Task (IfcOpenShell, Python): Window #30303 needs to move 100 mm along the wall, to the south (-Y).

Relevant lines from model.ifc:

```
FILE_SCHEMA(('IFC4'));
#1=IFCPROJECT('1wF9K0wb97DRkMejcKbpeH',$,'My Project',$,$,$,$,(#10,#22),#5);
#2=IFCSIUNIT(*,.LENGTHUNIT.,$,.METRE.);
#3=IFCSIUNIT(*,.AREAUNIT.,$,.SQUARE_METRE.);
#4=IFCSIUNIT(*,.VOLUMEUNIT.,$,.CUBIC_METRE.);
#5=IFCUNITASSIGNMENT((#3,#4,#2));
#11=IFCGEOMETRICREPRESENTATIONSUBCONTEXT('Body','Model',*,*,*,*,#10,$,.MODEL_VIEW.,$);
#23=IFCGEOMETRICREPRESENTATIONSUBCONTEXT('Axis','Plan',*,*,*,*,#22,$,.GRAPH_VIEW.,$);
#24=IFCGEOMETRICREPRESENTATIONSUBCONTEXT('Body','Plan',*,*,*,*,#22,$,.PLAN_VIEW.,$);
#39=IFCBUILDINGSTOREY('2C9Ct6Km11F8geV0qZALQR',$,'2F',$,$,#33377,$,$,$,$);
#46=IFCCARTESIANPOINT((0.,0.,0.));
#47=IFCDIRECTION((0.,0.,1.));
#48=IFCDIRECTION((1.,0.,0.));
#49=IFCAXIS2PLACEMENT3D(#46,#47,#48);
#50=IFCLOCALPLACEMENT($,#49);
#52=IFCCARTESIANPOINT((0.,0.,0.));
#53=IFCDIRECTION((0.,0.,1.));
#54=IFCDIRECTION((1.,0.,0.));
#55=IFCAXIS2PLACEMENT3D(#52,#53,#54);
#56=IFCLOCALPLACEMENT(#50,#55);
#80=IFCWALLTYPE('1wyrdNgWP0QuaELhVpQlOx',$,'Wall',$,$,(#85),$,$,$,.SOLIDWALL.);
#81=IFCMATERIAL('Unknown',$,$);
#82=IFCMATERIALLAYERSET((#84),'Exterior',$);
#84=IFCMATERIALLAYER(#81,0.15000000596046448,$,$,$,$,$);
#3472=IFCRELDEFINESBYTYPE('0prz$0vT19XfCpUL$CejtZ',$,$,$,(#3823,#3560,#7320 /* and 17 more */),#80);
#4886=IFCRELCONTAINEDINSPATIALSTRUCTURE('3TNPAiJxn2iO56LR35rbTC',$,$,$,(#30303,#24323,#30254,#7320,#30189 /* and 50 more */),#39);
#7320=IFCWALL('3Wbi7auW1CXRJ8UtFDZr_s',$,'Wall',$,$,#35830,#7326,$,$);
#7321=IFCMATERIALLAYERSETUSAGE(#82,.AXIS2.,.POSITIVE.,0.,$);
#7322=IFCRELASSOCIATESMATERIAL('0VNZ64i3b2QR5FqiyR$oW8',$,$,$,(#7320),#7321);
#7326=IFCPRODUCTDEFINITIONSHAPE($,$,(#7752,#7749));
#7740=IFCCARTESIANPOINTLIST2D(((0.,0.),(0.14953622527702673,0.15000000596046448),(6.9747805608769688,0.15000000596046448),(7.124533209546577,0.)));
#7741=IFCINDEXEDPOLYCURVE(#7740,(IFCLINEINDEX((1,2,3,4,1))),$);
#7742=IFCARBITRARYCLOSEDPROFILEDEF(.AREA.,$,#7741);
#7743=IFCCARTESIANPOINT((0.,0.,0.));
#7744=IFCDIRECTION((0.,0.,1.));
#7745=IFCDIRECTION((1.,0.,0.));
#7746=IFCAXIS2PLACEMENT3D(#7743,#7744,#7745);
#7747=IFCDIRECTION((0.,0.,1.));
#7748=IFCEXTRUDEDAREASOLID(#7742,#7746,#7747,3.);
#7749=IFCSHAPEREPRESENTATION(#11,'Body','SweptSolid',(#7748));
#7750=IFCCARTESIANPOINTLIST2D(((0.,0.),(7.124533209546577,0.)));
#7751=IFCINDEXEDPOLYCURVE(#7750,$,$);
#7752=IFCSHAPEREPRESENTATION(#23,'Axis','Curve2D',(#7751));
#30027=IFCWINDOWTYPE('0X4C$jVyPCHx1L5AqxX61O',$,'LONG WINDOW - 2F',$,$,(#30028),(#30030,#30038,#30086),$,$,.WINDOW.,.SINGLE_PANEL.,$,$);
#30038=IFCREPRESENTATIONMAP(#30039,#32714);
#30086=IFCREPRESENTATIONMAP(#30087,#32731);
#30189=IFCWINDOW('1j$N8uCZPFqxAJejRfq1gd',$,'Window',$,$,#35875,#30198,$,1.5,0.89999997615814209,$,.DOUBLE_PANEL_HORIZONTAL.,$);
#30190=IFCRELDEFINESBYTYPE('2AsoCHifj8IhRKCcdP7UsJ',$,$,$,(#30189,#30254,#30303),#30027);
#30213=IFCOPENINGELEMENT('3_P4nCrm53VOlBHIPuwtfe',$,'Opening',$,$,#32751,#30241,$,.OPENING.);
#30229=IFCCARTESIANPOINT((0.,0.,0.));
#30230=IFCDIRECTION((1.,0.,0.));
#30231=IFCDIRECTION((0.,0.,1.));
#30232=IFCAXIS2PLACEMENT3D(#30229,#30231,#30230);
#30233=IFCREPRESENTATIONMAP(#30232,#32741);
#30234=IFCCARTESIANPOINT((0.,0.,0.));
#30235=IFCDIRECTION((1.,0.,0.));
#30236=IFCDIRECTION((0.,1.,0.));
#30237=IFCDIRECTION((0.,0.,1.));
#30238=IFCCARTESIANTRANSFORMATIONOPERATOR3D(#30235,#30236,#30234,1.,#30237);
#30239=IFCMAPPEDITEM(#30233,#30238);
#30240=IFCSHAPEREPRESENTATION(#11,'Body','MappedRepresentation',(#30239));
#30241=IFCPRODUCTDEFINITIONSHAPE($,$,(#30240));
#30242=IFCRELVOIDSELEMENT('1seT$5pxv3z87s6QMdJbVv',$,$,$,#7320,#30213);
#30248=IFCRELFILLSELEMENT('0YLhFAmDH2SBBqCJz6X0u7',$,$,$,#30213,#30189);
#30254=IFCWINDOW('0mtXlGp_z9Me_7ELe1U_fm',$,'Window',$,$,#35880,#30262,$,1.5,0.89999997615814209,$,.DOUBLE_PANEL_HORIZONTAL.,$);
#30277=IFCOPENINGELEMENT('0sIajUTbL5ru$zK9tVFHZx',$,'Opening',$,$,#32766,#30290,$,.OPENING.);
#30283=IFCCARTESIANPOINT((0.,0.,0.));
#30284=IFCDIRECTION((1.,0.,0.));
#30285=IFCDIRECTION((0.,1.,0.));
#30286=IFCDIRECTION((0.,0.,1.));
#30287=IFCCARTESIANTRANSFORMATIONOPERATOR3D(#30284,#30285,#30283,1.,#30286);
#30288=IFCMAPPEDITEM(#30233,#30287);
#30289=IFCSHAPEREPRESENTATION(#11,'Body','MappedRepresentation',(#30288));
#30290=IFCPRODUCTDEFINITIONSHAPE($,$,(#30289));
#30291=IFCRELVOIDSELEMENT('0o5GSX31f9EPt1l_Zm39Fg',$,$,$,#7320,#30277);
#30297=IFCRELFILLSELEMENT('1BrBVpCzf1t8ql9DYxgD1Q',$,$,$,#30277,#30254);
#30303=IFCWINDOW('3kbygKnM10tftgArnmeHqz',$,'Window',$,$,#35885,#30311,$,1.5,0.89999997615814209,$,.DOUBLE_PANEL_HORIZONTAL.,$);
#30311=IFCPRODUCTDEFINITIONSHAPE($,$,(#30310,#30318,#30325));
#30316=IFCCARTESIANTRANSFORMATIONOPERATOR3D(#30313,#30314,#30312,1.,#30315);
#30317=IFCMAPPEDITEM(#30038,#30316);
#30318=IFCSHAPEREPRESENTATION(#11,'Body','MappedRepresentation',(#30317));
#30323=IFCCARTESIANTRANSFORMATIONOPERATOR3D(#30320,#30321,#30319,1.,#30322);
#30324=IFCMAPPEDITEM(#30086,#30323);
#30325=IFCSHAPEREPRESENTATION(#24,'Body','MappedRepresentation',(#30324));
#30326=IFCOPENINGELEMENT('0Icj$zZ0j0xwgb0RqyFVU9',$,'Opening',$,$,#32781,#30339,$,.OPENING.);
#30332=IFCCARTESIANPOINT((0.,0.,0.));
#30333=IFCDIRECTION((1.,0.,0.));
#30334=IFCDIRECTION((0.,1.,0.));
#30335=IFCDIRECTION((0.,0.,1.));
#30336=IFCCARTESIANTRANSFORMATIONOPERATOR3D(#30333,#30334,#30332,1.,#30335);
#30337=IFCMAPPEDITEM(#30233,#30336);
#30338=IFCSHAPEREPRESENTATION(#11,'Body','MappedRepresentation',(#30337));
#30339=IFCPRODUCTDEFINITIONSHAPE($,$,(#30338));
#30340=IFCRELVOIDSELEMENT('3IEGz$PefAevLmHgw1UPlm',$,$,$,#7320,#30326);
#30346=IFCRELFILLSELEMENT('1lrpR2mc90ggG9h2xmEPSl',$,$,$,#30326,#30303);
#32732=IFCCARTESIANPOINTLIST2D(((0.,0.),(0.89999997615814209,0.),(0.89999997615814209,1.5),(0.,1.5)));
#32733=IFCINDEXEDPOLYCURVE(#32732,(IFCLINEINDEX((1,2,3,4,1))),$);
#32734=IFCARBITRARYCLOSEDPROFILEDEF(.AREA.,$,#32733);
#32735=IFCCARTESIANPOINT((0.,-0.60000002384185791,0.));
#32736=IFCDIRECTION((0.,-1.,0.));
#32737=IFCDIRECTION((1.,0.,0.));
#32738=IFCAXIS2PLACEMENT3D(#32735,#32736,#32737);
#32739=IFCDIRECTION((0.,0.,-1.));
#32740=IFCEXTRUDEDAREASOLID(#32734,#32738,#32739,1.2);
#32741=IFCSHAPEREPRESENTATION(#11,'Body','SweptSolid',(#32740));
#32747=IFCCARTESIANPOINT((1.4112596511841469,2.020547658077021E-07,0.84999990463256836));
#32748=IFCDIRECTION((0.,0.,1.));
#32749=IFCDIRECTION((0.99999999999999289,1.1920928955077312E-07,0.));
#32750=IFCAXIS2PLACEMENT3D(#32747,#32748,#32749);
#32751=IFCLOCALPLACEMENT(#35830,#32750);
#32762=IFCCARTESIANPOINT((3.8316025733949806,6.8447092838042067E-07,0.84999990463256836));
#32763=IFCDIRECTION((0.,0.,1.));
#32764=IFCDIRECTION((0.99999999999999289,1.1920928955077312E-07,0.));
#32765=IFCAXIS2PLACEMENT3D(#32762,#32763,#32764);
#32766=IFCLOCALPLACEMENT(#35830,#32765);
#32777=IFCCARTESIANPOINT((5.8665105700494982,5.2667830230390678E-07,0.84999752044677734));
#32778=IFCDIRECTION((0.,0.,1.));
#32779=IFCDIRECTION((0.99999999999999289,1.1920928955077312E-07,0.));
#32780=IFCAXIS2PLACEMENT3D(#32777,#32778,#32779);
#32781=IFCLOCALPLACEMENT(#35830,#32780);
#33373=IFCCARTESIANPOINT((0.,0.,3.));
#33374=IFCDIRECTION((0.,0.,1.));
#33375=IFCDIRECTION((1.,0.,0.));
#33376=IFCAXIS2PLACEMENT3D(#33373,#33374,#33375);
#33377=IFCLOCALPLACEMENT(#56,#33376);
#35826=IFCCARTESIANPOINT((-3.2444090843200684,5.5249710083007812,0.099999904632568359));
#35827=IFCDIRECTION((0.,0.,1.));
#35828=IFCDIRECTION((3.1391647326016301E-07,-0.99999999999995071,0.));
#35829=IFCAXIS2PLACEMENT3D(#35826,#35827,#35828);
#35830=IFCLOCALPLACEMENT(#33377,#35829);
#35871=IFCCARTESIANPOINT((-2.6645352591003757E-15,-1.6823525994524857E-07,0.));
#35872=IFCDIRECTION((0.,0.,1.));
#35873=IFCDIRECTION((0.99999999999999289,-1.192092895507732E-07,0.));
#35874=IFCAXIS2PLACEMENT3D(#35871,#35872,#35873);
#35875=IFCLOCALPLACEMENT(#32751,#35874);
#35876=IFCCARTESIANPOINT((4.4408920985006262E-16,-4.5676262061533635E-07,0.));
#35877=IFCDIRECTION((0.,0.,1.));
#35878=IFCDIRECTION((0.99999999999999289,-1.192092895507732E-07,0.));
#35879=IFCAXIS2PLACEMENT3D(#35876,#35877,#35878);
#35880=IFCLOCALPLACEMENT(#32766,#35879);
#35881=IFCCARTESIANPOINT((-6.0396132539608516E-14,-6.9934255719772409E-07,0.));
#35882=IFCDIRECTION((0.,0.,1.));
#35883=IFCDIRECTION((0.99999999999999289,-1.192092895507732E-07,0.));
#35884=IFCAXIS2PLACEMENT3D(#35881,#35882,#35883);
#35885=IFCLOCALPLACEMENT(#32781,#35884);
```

```python
import ifcopenshell
import ifcopenshell.api.geometry
import ifcopenshell.util.placement
import ifcopenshell.util.unit

model = ifcopenshell.open("model.ifc")
unit_scale = ifcopenshell.util.unit.calculate_unit_scale(model)

window = model.by_id(30303)
opening = window.FillsVoids[0].RelatingOpeningElement
wall = opening.VoidsElements[0].RelatingBuildingElement

wall_matrix = ifcopenshell.util.placement.get_local_placement(wall.ObjectPlacement)
shift = wall_matrix[:3, 0] * 0.1 / unit_scale
before = ifcopenshell.util.placement.get_local_placement(window.ObjectPlacement)[:3, 3].copy()

# The window is placed relative to its opening, so it follows when the opening moves.
matrix = ifcopenshell.util.placement.get_local_placement(opening.ObjectPlacement)
matrix[:3, 3] += shift
ifcopenshell.api.geometry.edit_object_placement(
    model, product=opening, matrix=matrix, is_si=False, should_transform_children=True
)

after = ifcopenshell.util.placement.get_local_placement(window.ObjectPlacement)[:3, 3]
print("window moved by", (after - before).round(3) + 0.0)

model.write("model_updated.ifc")
```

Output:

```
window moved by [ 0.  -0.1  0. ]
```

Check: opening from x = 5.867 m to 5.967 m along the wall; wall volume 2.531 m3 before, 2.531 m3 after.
